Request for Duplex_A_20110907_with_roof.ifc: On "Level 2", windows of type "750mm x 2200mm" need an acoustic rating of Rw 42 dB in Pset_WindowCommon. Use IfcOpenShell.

First a look at what the model holds.

```python
import ifcopenshell
import ifcopenshell.util.element

model = ifcopenshell.open("Duplex_A_20110907_with_roof.ifc")
print(model.schema)
storey = next(s for s in model.by_type("IfcBuildingStorey") if s.Name == "Level 2")
windows = [e for e in ifcopenshell.util.element.get_decomposition(storey) if e.is_a("IfcWindow")]
seen = {}
for e in windows:
    element_type = ifcopenshell.util.element.get_type(e)
    key = (element_type.Name if element_type != e and element_type else None, ifcopenshell.util.element.get_pset(e, "Pset_WindowCommon", "AcousticRating"))
    seen[key] = seen.get(key, 0) + 1
for (name, value), count in sorted(seen.items(), key=str):
    print(count, "x", name, "|", value)
```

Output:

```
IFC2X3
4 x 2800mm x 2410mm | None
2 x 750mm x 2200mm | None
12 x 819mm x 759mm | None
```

```python
import ifcopenshell
import ifcopenshell.api.pset
import ifcopenshell.util.element

model = ifcopenshell.open("Duplex_A_20110907_with_roof.ifc")

storey = next(s for s in model.by_type("IfcBuildingStorey") if s.Name == "Level 2")
windows = [e for e in ifcopenshell.util.element.get_decomposition(storey) if e.is_a("IfcWindow")]

count = 0
for e in windows:
    element_type = ifcopenshell.util.element.get_type(e)
    if element_type in (None, e) or element_type.Name != "750mm x 2200mm":
        continue
    # add_pset returns the element's existing set when there is one.
    pset = ifcopenshell.api.pset.add_pset(model, product=e, name="Pset_WindowCommon")
    ifcopenshell.api.pset.edit_pset(model, pset=pset, properties={"AcousticRating": "Rw 42 dB"})
    count += 1

print(count, "windows updated")

model.write("Duplex_A_20110907_with_roof_rev.ifc")
```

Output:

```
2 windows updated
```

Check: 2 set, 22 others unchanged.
